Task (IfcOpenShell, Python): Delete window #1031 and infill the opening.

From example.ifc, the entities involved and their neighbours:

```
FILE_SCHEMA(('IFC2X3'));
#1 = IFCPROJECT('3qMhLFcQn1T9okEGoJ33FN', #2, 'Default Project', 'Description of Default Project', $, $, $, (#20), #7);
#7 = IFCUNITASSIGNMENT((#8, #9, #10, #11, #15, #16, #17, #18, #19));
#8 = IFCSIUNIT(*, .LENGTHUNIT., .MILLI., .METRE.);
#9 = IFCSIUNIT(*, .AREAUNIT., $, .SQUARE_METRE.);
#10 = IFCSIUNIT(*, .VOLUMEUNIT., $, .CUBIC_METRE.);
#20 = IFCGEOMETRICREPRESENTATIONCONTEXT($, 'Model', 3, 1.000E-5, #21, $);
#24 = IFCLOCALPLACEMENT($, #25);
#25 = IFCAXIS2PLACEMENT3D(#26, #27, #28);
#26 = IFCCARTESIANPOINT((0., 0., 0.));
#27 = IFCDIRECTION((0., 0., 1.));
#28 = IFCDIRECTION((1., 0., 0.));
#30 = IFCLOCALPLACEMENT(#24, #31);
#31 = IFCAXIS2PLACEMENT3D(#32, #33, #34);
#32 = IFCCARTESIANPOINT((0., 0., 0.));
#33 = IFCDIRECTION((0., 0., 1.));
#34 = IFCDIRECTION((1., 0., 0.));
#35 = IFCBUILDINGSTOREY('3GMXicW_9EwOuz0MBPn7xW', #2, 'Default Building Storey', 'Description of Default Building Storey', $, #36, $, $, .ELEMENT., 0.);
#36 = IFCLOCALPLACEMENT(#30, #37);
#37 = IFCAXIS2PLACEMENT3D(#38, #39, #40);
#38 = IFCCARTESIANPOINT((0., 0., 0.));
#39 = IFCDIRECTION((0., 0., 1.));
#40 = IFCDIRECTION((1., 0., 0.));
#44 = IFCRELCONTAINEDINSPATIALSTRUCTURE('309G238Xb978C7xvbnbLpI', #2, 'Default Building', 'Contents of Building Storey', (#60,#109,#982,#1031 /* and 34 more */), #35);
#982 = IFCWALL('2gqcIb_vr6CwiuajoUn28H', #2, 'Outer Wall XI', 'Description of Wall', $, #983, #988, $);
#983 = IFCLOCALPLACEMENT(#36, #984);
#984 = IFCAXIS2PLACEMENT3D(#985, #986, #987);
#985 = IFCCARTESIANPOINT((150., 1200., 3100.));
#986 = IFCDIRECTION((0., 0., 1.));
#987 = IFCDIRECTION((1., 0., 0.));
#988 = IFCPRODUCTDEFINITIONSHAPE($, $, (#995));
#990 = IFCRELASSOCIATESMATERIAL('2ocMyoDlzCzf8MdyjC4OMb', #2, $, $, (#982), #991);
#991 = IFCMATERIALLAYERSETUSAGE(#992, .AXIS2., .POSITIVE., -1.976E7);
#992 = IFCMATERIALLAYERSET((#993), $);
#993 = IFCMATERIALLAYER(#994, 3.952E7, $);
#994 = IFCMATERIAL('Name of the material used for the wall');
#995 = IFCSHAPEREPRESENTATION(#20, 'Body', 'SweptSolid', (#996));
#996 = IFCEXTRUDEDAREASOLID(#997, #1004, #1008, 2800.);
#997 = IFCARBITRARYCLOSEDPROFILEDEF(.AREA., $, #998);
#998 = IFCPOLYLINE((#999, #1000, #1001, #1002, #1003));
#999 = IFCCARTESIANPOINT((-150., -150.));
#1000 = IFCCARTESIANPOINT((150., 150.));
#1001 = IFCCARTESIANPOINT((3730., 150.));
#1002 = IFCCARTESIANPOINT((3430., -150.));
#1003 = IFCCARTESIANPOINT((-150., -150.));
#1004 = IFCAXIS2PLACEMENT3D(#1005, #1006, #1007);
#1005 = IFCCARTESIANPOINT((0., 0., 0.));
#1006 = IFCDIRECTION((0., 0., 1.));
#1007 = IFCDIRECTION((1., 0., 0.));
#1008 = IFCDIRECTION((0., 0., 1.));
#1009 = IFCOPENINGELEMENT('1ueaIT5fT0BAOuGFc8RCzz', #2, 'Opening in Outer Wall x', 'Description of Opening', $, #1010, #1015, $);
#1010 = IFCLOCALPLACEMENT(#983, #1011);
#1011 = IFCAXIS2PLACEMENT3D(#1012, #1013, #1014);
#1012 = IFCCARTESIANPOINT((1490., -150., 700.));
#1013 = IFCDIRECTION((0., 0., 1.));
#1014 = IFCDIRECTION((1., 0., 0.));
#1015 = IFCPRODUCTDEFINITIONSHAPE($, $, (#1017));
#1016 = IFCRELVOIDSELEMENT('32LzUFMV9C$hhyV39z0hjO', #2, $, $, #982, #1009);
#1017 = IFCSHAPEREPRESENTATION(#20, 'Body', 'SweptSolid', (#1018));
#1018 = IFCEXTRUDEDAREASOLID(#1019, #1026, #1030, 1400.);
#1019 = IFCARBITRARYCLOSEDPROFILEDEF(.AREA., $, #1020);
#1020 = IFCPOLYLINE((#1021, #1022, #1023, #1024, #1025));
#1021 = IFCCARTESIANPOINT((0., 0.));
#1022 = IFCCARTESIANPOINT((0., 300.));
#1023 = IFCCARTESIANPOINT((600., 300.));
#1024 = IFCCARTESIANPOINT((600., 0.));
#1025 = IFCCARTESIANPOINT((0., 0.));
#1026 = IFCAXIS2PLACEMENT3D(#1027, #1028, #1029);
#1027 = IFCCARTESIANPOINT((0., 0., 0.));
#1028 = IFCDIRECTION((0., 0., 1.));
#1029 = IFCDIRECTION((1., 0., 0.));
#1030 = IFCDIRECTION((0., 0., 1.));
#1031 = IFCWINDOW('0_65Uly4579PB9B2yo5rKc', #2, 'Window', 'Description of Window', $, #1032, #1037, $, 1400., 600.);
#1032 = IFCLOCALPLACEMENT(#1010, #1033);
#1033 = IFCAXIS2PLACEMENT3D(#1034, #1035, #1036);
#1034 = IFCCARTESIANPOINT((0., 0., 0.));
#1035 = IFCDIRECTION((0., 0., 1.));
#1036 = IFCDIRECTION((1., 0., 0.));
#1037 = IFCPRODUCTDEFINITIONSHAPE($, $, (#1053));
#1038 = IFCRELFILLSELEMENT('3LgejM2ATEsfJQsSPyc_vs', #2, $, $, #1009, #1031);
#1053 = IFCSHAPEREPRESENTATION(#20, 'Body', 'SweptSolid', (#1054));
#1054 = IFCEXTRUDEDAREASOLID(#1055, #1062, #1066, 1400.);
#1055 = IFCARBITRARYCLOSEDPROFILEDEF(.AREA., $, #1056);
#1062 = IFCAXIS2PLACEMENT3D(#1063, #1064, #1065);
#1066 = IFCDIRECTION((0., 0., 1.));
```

```python
import ifcopenshell
import ifcopenshell.api.feature
import ifcopenshell.api.root
import ifcopenshell.geom
import ifcopenshell.util.shape

model = ifcopenshell.open("example.ifc")
settings = ifcopenshell.geom.settings()


def volume(element):
    """Net volume in cubic metres, openings subtracted."""
    shape = ifcopenshell.geom.create_shape(settings, element)
    return ifcopenshell.util.shape.get_volume(shape.geometry)


window = model.by_guid("0_65Uly4579PB9B2yo5rKc")
opening = window.FillsVoids[0].RelatingOpeningElement
wall = opening.VoidsElements[0].RelatingBuildingElement
before = volume(wall)

ifcopenshell.api.root.remove_product(model, product=window)
ifcopenshell.api.feature.remove_feature(model, feature=opening)

after = volume(wall)

print(f"wall volume {before:.3f} -> {after:.3f} m3")

model.write("example_updated.ifc")
```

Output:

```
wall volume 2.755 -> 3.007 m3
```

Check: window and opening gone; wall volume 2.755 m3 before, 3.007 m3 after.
